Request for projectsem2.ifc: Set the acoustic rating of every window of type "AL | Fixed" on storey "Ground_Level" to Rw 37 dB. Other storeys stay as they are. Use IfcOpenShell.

First a look at what the model holds.

```python
import ifcopenshell
import ifcopenshell.util.element

model = ifcopenshell.open("projectsem2.ifc")
print(model.schema)
storey = next(s for s in model.by_type("IfcBuildingStorey") if s.Name == "Ground_Level")
windows = [e for e in ifcopenshell.util.element.get_decomposition(storey) if e.is_a("IfcWindow")]
seen = {}
for e in windows:
    element_type = ifcopenshell.util.element.get_type(e)
    key = (element_type.Name if element_type != e and element_type else None, ifcopenshell.util.element.get_pset(e, "Pset_WindowCommon", "AcousticRating"))
    seen[key] = seen.get(key, 0) + 1
for (name, value), count in sorted(seen.items(), key=str):
    print(count, "x", name, "|", value)
```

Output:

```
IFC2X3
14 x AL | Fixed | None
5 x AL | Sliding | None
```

```python
import ifcopenshell
import ifcopenshell.api.pset
import ifcopenshell.util.element

model = ifcopenshell.open("projectsem2.ifc")

storey = next(s for s in model.by_type("IfcBuildingStorey") if s.Name == "Ground_Level")
windows = [e for e in ifcopenshell.util.element.get_decomposition(storey) if e.is_a("IfcWindow")]

count = 0
for e in windows:
    element_type = ifcopenshell.util.element.get_type(e)
    if element_type in (None, e) or element_type.Name != "AL | Fixed":
        continue
    # add_pset returns the element's existing set when there is one.
    pset = ifcopenshell.api.pset.add_pset(model, product=e, name="Pset_WindowCommon")
    ifcopenshell.api.pset.edit_pset(model, pset=pset, properties={"AcousticRating": "Rw 37 dB"})
    count += 1

print(count, "windows updated")

model.write("projectsem2_edited.ifc")
```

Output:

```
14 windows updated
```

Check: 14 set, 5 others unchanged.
